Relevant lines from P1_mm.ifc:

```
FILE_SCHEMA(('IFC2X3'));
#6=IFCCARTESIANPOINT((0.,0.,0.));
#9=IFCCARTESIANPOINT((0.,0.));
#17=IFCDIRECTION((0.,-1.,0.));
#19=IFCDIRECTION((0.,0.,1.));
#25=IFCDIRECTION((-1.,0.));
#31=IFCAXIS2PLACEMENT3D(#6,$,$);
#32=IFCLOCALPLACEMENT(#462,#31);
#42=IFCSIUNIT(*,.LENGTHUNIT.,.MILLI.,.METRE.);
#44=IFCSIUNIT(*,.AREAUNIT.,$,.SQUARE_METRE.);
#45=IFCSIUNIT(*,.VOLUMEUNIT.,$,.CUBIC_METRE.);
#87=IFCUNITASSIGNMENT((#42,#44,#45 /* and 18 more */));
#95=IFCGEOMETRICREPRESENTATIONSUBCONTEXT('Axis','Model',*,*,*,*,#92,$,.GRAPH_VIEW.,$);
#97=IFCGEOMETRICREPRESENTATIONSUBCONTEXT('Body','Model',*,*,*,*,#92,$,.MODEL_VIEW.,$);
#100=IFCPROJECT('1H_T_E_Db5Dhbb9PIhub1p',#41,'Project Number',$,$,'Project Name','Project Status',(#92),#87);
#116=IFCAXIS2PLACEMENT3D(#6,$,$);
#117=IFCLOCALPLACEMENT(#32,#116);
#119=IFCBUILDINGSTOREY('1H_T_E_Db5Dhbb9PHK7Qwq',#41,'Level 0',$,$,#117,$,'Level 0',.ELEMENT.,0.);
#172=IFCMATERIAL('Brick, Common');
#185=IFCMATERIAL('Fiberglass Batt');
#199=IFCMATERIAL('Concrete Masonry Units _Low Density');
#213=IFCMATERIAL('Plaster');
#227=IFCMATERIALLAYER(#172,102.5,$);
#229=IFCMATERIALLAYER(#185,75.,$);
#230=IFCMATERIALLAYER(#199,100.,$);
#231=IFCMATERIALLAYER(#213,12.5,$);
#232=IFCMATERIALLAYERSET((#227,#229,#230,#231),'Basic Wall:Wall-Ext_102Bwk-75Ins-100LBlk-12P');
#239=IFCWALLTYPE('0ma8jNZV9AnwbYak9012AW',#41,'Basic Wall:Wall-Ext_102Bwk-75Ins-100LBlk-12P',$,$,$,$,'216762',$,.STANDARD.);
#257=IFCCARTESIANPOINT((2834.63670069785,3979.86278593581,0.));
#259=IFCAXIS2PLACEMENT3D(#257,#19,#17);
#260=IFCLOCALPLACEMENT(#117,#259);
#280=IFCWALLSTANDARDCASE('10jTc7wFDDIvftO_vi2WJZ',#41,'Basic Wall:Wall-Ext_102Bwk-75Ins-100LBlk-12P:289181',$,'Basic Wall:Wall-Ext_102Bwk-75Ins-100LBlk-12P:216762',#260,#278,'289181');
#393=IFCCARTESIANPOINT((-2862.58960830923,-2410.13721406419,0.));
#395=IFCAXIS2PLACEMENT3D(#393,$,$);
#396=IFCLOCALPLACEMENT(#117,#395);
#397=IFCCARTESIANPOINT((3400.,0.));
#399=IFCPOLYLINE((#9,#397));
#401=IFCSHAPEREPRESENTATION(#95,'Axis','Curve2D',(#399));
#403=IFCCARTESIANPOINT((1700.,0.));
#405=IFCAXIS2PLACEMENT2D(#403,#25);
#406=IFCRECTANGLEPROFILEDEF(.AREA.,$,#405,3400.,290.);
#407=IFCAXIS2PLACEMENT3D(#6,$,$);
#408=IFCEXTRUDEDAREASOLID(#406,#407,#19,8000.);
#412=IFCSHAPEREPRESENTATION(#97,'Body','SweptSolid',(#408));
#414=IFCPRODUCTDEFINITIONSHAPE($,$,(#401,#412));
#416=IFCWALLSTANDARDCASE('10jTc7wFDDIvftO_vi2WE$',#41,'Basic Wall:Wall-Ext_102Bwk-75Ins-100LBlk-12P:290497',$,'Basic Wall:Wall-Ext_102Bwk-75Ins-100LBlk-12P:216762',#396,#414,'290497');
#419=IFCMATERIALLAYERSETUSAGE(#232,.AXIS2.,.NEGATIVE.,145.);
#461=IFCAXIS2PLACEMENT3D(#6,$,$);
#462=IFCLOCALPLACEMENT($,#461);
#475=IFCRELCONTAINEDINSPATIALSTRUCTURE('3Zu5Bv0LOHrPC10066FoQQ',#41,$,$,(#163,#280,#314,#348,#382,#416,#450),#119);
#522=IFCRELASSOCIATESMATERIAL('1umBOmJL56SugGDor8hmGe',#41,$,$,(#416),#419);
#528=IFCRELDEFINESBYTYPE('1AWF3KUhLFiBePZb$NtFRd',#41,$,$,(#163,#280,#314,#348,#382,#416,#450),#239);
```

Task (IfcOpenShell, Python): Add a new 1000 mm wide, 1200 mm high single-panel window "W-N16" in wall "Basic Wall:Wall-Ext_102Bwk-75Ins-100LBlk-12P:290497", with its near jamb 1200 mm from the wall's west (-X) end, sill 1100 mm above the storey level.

```python
import numpy as np
import ifcopenshell
import ifcopenshell.api.feature
import ifcopenshell.api.geometry
import ifcopenshell.api.root
import ifcopenshell.api.spatial
import ifcopenshell.api.type
import ifcopenshell.geom
import ifcopenshell.util.element
import ifcopenshell.util.placement
import ifcopenshell.util.representation
import ifcopenshell.util.shape
import ifcopenshell.util.unit

model = ifcopenshell.open("P1_mm.ifc")
unit_scale = ifcopenshell.util.unit.calculate_unit_scale(model)
settings = ifcopenshell.geom.settings()


def volume(element):
    """Net volume in cubic metres, openings subtracted."""
    shape = ifcopenshell.geom.create_shape(settings, element)
    return ifcopenshell.util.shape.get_volume(shape.geometry)


wall = model.by_id(416)
storey = ifcopenshell.util.element.get_container(wall, ifc_class="IfcBuildingStorey")
context = ifcopenshell.util.representation.get_context(model, "Model", "Body", "MODEL_VIEW")
before = volume(wall)

width, height, from_end, sill = 1, 1.2, 1.2, 1.1  # metres

# The wall runs along its own X axis, and the end named is its -X end.
wall_shape = ifcopenshell.geom.create_shape(settings, wall)
x, y, z = ifcopenshell.util.shape.get_vertices(wall_shape.geometry).T
start = x.min() + from_end
face, thickness = float(y.min()), float(y.max() - y.min())
wall_matrix = ifcopenshell.util.placement.get_local_placement(wall.ObjectPlacement)
level = ifcopenshell.util.placement.get_local_placement(storey.ObjectPlacement)[2, 3]


def in_wall(x, y):
    """Placement at x, y metres in the wall's axes, at sill height."""
    matrix = wall_matrix.copy()
    matrix[:, 3] = wall_matrix @ np.array([x / unit_scale, y / unit_scale, 0.0, 1.0])
    matrix[2, 3] = level + sill / unit_scale
    return matrix


# Opening: a box that overshoots both wall faces by 50 mm.
opening = ifcopenshell.api.root.create_entity(model, ifc_class="IfcOpeningElement")
box = ifcopenshell.api.geometry.add_wall_representation(
    model, context=context, length=width, height=height, thickness=thickness + 0.1
)
ifcopenshell.api.geometry.assign_representation(model, product=opening, representation=box)
ifcopenshell.api.geometry.edit_object_placement(model, product=opening, matrix=in_wall(start, face - 0.05), is_si=False)
ifcopenshell.api.feature.add_feature(model, feature=opening, element=wall)

window = ifcopenshell.api.root.create_entity(model, ifc_class="IfcWindow", name="W-N16")
window.OverallWidth, window.OverallHeight = width / unit_scale, height / unit_scale
body = ifcopenshell.api.geometry.add_window_representation(
    model,
    context=context,
    overall_width=window.OverallWidth,
    overall_height=window.OverallHeight,
    partition_type="SINGLE_PANEL",
)
ifcopenshell.api.geometry.assign_representation(model, product=window, representation=body)
ifcopenshell.api.spatial.assign_container(model, products=[window], relating_structure=storey)
fills = ifcopenshell.api.feature.add_filling(model, opening=opening, element=window)
fills.OwnerHistory = window.OwnerHistory  # required in IFC2X3

# IFC2X3 keeps the operation on the window style.
style = ifcopenshell.api.root.create_entity(model, ifc_class="IfcWindowStyle", name="W-N16")
style.OperationType, style.ConstructionType = "SINGLE_PANEL", "NOTDEFINED"
style.ParameterTakesPrecedence = style.Sizeable = False
ifcopenshell.api.type.assign_type(model, related_objects=[window], relating_type=style)

# Centre the window in the wall's thickness.
ifcopenshell.api.geometry.edit_object_placement(model, product=window, matrix=in_wall(start, face), is_si=False)
window_shape = ifcopenshell.geom.create_shape(settings, window)
depth = ifcopenshell.util.shape.get_vertices(window_shape.geometry)[:, 1]
offset = face + thickness / 2 - (depth.min() + depth.max()) / 2
ifcopenshell.api.geometry.edit_object_placement(model, product=window, matrix=in_wall(start, offset), is_si=False)

after = volume(wall)

print(f"wall volume {before:.3f} -> {after:.3f} m3")

model.write("P1_mm_v2.ifc")
```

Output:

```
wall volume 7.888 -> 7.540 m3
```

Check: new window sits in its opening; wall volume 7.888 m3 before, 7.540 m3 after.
